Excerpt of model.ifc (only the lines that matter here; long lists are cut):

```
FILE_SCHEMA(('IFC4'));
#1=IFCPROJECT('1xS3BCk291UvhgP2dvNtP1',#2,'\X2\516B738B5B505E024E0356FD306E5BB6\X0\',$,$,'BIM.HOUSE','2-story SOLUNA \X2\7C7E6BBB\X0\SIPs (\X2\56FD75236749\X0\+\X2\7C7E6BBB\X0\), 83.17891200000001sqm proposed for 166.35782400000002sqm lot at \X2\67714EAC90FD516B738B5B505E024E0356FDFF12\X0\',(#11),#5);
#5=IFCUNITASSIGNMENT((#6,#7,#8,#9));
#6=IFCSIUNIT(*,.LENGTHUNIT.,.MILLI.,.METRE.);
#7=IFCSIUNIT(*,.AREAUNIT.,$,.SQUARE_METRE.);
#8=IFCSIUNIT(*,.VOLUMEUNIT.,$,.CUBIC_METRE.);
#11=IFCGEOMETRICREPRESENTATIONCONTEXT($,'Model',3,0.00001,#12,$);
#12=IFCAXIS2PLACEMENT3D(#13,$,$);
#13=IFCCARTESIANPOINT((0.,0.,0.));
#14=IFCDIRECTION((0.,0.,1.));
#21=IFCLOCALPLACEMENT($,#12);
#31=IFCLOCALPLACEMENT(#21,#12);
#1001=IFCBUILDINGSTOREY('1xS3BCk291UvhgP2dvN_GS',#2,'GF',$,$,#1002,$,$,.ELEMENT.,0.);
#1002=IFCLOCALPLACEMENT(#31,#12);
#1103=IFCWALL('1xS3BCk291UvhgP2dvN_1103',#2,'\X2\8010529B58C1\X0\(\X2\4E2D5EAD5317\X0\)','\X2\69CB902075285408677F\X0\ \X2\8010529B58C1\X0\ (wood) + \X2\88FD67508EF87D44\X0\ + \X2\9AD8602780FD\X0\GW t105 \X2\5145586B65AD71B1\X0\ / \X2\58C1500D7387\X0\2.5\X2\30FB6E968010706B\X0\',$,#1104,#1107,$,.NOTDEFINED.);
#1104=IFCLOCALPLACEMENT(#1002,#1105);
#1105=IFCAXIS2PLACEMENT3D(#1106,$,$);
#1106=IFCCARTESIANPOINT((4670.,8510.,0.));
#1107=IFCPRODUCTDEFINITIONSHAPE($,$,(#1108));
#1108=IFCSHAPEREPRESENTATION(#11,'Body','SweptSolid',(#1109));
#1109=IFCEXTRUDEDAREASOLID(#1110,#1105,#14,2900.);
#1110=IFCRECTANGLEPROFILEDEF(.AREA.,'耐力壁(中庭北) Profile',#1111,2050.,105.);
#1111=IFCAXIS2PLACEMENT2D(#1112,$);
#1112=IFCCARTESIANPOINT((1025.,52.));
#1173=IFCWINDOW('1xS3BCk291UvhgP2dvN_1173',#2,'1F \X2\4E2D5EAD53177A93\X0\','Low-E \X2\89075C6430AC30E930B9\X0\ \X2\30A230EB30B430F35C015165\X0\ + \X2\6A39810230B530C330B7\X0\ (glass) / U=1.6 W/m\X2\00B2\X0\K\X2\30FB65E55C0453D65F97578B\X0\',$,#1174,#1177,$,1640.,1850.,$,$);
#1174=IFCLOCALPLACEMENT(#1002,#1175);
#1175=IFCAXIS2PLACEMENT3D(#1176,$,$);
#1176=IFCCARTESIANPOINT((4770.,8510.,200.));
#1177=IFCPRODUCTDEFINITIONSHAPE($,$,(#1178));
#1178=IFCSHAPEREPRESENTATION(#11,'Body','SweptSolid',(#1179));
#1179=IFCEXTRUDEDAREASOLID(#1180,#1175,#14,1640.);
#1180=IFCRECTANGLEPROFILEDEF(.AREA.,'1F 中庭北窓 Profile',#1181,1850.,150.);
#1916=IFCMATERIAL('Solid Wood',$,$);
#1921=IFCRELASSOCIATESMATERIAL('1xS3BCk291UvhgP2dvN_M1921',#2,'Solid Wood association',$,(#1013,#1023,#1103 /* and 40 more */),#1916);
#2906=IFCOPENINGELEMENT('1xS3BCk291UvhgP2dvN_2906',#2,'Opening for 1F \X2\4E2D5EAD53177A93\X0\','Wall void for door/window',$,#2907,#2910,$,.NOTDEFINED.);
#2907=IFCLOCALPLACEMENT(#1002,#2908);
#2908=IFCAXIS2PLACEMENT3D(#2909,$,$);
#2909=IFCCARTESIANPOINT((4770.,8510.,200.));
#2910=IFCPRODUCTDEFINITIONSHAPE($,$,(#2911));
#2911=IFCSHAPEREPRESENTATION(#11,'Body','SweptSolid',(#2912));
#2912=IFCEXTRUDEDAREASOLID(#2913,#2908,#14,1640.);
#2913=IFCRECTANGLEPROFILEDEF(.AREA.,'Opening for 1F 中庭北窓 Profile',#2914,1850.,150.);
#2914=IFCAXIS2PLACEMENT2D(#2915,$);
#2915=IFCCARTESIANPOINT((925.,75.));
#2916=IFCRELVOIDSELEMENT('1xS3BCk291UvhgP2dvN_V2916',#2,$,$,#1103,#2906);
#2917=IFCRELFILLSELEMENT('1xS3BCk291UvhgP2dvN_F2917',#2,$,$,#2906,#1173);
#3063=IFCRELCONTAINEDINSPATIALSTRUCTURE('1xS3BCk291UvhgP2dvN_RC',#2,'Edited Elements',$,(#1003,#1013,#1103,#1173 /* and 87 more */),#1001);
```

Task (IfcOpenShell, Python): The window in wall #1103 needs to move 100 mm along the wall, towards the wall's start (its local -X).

```python
import ifcopenshell
import ifcopenshell.api.geometry
import ifcopenshell.util.placement
import ifcopenshell.util.unit

model = ifcopenshell.open("model.ifc")
unit_scale = ifcopenshell.util.unit.calculate_unit_scale(model)

window = model.by_guid("1xS3BCk291UvhgP2dvN_1173")
opening = window.FillsVoids[0].RelatingOpeningElement
wall = opening.VoidsElements[0].RelatingBuildingElement

wall_matrix = ifcopenshell.util.placement.get_local_placement(wall.ObjectPlacement)
shift = wall_matrix[:3, 0] * -0.1 / unit_scale
before = ifcopenshell.util.placement.get_local_placement(window.ObjectPlacement)[:3, 3].copy()

# The window is not placed relative to its opening, so move both.
for product in (opening, window):
    matrix = ifcopenshell.util.placement.get_local_placement(product.ObjectPlacement)
    matrix[:3, 3] += shift
    ifcopenshell.api.geometry.edit_object_placement(model, product=product, matrix=matrix, is_si=False)

after = ifcopenshell.util.placement.get_local_placement(window.ObjectPlacement)[:3, 3]
print("window moved by", (after - before).round(3) + 0.0)

model.write("model_edited.ifc")
```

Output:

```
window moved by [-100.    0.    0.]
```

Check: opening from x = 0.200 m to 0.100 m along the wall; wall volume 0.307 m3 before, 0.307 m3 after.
